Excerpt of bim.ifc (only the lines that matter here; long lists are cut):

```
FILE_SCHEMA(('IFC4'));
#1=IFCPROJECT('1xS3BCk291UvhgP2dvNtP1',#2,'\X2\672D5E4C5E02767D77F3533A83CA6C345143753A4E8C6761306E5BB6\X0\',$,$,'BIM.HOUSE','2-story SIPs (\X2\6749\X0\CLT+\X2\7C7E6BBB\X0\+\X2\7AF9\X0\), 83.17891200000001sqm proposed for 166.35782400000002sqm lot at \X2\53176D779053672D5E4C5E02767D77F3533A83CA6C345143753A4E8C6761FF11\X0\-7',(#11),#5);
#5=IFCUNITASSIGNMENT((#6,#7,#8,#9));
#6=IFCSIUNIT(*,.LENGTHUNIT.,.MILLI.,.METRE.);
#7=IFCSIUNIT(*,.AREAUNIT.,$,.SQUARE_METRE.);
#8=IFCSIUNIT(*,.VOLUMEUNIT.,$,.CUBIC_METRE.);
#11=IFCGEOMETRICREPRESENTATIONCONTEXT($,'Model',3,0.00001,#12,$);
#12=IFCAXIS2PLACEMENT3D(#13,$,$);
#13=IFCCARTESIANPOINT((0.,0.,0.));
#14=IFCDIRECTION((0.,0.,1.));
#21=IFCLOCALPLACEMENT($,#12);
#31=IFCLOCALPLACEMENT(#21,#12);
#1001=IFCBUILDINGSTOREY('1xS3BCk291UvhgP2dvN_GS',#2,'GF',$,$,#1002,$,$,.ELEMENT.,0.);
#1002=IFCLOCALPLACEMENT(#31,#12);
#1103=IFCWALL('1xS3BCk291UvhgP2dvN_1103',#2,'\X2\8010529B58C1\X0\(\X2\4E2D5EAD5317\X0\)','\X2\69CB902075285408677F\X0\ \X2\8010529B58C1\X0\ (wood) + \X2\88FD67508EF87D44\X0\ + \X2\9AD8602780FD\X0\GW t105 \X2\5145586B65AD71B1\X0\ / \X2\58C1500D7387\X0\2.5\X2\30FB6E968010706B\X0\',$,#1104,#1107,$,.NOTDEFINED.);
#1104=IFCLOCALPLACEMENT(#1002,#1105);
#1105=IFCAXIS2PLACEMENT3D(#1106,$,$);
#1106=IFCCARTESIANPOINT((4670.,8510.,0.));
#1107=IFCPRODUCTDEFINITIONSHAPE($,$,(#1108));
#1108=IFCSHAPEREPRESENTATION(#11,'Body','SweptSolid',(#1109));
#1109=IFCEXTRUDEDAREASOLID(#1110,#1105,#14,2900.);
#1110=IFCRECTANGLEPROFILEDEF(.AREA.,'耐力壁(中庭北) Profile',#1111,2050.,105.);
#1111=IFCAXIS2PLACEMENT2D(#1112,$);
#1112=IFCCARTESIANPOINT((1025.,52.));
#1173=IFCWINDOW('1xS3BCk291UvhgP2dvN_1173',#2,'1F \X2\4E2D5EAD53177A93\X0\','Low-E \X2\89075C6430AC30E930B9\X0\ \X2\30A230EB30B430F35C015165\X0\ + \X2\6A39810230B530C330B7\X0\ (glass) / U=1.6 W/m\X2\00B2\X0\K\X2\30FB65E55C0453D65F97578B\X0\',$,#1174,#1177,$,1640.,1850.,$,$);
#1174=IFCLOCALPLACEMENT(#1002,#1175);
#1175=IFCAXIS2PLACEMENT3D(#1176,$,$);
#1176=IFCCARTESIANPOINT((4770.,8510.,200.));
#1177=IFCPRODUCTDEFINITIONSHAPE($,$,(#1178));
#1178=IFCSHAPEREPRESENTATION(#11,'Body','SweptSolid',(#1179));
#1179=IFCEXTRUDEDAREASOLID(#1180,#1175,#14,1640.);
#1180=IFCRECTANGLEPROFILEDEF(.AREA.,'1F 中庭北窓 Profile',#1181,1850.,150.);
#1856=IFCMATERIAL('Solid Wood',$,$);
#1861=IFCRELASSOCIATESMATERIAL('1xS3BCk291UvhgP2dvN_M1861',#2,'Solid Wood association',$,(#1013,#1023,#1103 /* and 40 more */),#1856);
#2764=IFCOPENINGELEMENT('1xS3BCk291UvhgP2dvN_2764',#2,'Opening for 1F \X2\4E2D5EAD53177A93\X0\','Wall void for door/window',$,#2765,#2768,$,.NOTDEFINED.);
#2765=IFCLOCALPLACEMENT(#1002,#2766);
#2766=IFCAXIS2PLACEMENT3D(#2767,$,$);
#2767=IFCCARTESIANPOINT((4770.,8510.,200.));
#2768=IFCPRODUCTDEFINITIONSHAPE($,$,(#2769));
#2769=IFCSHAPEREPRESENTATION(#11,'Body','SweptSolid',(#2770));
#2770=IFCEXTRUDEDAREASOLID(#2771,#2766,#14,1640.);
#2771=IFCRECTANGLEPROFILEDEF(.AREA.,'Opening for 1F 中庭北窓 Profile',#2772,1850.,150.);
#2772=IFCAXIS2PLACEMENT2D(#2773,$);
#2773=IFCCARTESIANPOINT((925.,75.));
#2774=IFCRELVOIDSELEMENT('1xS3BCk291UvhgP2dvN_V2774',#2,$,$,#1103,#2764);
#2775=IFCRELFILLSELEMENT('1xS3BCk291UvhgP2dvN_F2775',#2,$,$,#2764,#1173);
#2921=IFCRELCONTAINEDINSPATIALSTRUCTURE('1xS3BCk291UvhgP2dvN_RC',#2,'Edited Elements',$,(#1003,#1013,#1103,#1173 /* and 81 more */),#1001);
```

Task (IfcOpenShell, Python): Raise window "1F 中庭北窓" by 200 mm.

```python
import numpy as np
import ifcopenshell
import ifcopenshell.api.geometry
import ifcopenshell.util.placement
import ifcopenshell.util.unit

model = ifcopenshell.open("bim.ifc")
unit_scale = ifcopenshell.util.unit.calculate_unit_scale(model)

window = model.by_id(1173)
opening = window.FillsVoids[0].RelatingOpeningElement
dz = 200.0

shift = np.array([0.0, 0.0, dz])
# The window is not placed relative to its opening, so move both.
for product in (opening, window):
    matrix = ifcopenshell.util.placement.get_local_placement(product.ObjectPlacement)
    matrix[:3, 3] += shift
    ifcopenshell.api.geometry.edit_object_placement(model, product=product, matrix=matrix, is_si=False)

print(f"moved by {dz * unit_scale:+.3f} m")

model.write("bim-out.ifc")
```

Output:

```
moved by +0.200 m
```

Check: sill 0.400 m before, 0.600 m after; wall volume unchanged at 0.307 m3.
